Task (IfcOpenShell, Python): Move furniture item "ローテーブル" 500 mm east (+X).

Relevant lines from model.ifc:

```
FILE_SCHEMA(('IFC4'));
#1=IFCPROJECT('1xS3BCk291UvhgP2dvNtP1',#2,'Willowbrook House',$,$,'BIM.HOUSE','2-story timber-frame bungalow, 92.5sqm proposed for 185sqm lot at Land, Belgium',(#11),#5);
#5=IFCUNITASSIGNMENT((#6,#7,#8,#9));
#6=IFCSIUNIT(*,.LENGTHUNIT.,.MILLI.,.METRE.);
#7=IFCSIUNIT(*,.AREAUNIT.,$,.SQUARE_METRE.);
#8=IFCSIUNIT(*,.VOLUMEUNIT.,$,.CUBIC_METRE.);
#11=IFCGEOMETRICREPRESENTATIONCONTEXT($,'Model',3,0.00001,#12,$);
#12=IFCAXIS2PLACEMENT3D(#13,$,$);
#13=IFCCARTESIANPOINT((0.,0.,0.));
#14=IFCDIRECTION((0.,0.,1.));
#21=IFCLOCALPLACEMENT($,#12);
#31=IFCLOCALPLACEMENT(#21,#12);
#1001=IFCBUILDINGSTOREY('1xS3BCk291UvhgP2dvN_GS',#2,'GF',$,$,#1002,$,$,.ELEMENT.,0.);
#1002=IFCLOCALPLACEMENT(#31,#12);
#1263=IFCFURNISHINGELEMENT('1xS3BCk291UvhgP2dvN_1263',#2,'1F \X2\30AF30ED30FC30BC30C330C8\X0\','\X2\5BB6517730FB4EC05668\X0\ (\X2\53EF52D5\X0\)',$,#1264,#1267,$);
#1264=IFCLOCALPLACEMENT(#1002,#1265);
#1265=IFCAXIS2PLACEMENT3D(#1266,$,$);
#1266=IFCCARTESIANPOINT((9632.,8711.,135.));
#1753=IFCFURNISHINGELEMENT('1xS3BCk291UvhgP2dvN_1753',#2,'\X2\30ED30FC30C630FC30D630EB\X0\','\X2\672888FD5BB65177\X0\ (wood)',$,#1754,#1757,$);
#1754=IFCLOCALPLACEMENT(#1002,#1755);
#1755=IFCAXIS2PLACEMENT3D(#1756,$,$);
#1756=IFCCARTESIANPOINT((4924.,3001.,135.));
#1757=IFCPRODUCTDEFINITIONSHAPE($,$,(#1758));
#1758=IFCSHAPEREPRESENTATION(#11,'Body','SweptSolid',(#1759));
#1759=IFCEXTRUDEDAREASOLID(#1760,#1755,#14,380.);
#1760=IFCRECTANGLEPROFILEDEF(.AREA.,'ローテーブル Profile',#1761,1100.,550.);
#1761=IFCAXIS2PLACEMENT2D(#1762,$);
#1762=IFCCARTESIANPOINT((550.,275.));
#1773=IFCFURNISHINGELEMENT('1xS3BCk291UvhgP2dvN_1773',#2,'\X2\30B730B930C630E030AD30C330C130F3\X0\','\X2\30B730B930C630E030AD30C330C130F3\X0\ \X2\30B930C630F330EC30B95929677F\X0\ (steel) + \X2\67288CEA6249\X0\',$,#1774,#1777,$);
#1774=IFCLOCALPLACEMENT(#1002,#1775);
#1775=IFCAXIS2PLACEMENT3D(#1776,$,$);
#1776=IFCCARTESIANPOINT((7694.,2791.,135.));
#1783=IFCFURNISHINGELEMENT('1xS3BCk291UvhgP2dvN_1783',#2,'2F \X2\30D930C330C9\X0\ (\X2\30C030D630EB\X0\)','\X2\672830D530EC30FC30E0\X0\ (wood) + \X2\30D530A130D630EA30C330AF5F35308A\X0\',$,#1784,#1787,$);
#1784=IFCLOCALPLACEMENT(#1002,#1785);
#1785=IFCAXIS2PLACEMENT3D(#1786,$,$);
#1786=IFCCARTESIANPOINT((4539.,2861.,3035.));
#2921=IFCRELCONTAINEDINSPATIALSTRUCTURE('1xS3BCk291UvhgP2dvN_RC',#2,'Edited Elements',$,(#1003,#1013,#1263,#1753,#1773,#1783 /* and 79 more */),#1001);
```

```python
import ifcopenshell
import ifcopenshell.api.geometry
import ifcopenshell.util.placement
import ifcopenshell.util.unit

model = ifcopenshell.open("model.ifc")
unit_scale = ifcopenshell.util.unit.calculate_unit_scale(model)

item = model.by_guid("1xS3BCk291UvhgP2dvN_1753")
matrix = ifcopenshell.util.placement.get_local_placement(item.ObjectPlacement)
matrix[0, 3] += 0.5 / unit_scale
ifcopenshell.api.geometry.edit_object_placement(model, product=item, matrix=matrix, is_si=False)

print(ifcopenshell.util.placement.get_local_placement(item.ObjectPlacement).round(3) + 0.0)

model.write("model_v2.ifc")
```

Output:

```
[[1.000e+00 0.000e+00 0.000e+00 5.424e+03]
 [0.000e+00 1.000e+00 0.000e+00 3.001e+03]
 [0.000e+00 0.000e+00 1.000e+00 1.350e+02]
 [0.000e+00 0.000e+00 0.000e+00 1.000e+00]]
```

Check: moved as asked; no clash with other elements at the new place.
